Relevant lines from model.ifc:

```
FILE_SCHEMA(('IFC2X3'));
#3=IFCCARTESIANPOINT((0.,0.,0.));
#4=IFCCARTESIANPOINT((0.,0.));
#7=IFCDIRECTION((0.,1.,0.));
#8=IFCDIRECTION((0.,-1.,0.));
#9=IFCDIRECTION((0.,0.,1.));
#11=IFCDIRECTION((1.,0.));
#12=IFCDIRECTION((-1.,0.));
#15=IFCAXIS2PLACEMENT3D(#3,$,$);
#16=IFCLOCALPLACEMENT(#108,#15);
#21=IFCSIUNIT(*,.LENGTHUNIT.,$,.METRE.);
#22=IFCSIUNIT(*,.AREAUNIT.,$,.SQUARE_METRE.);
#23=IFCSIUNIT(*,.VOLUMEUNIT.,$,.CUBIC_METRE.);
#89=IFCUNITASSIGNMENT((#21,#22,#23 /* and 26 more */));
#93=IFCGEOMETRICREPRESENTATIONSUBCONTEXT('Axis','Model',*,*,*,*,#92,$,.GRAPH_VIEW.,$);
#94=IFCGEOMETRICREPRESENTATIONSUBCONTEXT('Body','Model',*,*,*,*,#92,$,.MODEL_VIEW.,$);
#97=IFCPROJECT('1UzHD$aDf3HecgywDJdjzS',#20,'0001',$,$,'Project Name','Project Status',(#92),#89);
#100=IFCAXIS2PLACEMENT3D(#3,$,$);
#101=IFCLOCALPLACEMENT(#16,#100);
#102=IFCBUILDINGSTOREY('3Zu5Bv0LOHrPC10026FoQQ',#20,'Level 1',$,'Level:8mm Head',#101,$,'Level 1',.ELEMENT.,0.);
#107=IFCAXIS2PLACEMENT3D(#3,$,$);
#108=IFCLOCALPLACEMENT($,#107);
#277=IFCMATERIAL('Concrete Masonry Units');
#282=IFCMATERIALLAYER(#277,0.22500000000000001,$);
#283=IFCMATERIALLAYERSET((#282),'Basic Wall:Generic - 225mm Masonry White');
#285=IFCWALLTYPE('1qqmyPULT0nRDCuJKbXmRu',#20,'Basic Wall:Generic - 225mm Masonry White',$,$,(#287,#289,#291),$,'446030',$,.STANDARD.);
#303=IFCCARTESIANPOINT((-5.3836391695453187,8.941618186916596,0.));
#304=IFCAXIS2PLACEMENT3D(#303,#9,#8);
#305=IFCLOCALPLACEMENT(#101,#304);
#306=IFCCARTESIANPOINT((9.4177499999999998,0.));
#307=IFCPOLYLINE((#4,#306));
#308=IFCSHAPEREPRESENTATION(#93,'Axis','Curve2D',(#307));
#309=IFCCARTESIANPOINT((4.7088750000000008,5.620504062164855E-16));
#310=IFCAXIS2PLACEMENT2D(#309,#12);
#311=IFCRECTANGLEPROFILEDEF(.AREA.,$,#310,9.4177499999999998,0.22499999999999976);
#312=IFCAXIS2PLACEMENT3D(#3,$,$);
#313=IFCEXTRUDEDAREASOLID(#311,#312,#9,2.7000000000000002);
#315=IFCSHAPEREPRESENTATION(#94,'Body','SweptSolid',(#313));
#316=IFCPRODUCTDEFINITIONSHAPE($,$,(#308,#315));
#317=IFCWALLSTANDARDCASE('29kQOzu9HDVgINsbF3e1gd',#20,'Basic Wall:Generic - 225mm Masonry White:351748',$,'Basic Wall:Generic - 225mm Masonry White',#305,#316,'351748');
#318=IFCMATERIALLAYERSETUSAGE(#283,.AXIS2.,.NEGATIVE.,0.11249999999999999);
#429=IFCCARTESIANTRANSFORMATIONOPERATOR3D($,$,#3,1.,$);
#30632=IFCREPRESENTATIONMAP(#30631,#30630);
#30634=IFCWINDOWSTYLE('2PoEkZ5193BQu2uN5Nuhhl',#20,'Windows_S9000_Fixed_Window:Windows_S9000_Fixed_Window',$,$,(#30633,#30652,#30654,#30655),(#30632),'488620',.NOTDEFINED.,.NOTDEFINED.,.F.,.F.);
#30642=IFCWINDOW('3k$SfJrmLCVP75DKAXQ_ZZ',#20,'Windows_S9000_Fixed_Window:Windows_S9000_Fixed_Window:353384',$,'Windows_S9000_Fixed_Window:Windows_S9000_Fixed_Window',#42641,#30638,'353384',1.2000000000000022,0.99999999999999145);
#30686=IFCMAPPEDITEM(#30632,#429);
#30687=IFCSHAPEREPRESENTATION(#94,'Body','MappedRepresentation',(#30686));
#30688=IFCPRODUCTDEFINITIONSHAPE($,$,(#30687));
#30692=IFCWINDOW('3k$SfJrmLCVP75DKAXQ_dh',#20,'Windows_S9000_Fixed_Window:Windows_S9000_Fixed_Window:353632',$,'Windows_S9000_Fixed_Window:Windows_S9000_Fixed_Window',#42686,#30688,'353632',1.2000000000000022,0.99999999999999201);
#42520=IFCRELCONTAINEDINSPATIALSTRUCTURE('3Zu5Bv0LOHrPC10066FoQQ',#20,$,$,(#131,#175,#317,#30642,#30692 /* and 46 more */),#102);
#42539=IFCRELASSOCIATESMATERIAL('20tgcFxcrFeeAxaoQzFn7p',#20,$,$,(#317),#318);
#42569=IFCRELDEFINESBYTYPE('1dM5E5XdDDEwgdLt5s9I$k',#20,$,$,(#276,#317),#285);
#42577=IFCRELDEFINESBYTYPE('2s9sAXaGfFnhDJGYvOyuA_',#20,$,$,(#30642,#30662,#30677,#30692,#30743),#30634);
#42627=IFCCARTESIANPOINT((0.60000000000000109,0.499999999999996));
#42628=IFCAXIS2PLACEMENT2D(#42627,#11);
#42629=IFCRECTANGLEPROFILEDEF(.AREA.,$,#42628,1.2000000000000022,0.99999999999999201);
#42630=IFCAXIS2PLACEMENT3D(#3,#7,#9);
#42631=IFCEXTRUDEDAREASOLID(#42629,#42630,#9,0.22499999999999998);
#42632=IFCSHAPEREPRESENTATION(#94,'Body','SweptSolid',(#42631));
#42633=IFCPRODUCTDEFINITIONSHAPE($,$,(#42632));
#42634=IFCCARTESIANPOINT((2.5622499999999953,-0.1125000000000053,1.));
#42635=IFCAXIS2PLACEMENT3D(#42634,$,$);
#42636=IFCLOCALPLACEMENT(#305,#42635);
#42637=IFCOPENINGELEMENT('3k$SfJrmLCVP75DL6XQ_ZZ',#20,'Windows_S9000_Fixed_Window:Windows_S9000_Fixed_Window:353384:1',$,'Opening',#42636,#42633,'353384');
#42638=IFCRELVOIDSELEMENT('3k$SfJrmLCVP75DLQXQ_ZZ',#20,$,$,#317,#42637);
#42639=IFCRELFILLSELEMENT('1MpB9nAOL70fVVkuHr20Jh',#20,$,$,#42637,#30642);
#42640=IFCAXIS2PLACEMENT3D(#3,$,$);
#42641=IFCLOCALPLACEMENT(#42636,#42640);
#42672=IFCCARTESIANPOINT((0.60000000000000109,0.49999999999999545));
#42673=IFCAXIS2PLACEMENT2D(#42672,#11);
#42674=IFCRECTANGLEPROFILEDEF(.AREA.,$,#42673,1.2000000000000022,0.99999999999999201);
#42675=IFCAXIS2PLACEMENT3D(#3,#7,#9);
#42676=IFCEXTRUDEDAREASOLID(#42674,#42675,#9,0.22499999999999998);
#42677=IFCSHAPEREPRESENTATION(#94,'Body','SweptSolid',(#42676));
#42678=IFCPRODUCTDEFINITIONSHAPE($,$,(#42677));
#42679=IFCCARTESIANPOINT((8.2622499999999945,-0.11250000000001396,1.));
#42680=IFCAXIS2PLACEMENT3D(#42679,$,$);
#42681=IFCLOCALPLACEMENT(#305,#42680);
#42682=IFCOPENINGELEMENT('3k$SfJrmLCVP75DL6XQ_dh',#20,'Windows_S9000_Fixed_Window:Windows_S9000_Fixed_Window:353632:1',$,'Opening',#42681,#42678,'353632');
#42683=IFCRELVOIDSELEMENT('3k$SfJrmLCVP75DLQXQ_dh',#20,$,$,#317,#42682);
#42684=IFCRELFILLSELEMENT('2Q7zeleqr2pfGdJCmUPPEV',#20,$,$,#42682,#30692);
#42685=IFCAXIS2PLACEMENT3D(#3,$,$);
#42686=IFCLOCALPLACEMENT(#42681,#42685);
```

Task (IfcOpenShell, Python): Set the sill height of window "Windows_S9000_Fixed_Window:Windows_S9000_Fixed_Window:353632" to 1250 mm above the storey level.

```python
import numpy as np
import ifcopenshell
import ifcopenshell.api.geometry
import ifcopenshell.geom
import ifcopenshell.util.element
import ifcopenshell.util.placement
import ifcopenshell.util.shape
import ifcopenshell.util.unit

model = ifcopenshell.open("model.ifc")
unit_scale = ifcopenshell.util.unit.calculate_unit_scale(model)

window = model.by_id(30692)
opening = window.FillsVoids[0].RelatingOpeningElement
storey = ifcopenshell.util.element.get_container(window, ifc_class="IfcBuildingStorey")
level = ifcopenshell.util.placement.get_local_placement(storey.ObjectPlacement)[2, 3]

# The opening's origin need not be at the sill, so measure its lowest point.
shape = ifcopenshell.geom.create_shape(ifcopenshell.geom.settings(), opening)
bottom = ifcopenshell.util.shape.get_shape_bottom_elevation(shape, shape.geometry) / unit_scale
dz = level + 1.25 - bottom

shift = np.array([0.0, 0.0, dz])
# The window is placed relative to its opening, so it follows when the opening moves.
matrix = ifcopenshell.util.placement.get_local_placement(opening.ObjectPlacement)
matrix[:3, 3] += shift
ifcopenshell.api.geometry.edit_object_placement(
    model, product=opening, matrix=matrix, is_si=False, should_transform_children=True
)

print(f"moved by {dz * unit_scale:+.3f} m")

model.write("model_updated.ifc")
```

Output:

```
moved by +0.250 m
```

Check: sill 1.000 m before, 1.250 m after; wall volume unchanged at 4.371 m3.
